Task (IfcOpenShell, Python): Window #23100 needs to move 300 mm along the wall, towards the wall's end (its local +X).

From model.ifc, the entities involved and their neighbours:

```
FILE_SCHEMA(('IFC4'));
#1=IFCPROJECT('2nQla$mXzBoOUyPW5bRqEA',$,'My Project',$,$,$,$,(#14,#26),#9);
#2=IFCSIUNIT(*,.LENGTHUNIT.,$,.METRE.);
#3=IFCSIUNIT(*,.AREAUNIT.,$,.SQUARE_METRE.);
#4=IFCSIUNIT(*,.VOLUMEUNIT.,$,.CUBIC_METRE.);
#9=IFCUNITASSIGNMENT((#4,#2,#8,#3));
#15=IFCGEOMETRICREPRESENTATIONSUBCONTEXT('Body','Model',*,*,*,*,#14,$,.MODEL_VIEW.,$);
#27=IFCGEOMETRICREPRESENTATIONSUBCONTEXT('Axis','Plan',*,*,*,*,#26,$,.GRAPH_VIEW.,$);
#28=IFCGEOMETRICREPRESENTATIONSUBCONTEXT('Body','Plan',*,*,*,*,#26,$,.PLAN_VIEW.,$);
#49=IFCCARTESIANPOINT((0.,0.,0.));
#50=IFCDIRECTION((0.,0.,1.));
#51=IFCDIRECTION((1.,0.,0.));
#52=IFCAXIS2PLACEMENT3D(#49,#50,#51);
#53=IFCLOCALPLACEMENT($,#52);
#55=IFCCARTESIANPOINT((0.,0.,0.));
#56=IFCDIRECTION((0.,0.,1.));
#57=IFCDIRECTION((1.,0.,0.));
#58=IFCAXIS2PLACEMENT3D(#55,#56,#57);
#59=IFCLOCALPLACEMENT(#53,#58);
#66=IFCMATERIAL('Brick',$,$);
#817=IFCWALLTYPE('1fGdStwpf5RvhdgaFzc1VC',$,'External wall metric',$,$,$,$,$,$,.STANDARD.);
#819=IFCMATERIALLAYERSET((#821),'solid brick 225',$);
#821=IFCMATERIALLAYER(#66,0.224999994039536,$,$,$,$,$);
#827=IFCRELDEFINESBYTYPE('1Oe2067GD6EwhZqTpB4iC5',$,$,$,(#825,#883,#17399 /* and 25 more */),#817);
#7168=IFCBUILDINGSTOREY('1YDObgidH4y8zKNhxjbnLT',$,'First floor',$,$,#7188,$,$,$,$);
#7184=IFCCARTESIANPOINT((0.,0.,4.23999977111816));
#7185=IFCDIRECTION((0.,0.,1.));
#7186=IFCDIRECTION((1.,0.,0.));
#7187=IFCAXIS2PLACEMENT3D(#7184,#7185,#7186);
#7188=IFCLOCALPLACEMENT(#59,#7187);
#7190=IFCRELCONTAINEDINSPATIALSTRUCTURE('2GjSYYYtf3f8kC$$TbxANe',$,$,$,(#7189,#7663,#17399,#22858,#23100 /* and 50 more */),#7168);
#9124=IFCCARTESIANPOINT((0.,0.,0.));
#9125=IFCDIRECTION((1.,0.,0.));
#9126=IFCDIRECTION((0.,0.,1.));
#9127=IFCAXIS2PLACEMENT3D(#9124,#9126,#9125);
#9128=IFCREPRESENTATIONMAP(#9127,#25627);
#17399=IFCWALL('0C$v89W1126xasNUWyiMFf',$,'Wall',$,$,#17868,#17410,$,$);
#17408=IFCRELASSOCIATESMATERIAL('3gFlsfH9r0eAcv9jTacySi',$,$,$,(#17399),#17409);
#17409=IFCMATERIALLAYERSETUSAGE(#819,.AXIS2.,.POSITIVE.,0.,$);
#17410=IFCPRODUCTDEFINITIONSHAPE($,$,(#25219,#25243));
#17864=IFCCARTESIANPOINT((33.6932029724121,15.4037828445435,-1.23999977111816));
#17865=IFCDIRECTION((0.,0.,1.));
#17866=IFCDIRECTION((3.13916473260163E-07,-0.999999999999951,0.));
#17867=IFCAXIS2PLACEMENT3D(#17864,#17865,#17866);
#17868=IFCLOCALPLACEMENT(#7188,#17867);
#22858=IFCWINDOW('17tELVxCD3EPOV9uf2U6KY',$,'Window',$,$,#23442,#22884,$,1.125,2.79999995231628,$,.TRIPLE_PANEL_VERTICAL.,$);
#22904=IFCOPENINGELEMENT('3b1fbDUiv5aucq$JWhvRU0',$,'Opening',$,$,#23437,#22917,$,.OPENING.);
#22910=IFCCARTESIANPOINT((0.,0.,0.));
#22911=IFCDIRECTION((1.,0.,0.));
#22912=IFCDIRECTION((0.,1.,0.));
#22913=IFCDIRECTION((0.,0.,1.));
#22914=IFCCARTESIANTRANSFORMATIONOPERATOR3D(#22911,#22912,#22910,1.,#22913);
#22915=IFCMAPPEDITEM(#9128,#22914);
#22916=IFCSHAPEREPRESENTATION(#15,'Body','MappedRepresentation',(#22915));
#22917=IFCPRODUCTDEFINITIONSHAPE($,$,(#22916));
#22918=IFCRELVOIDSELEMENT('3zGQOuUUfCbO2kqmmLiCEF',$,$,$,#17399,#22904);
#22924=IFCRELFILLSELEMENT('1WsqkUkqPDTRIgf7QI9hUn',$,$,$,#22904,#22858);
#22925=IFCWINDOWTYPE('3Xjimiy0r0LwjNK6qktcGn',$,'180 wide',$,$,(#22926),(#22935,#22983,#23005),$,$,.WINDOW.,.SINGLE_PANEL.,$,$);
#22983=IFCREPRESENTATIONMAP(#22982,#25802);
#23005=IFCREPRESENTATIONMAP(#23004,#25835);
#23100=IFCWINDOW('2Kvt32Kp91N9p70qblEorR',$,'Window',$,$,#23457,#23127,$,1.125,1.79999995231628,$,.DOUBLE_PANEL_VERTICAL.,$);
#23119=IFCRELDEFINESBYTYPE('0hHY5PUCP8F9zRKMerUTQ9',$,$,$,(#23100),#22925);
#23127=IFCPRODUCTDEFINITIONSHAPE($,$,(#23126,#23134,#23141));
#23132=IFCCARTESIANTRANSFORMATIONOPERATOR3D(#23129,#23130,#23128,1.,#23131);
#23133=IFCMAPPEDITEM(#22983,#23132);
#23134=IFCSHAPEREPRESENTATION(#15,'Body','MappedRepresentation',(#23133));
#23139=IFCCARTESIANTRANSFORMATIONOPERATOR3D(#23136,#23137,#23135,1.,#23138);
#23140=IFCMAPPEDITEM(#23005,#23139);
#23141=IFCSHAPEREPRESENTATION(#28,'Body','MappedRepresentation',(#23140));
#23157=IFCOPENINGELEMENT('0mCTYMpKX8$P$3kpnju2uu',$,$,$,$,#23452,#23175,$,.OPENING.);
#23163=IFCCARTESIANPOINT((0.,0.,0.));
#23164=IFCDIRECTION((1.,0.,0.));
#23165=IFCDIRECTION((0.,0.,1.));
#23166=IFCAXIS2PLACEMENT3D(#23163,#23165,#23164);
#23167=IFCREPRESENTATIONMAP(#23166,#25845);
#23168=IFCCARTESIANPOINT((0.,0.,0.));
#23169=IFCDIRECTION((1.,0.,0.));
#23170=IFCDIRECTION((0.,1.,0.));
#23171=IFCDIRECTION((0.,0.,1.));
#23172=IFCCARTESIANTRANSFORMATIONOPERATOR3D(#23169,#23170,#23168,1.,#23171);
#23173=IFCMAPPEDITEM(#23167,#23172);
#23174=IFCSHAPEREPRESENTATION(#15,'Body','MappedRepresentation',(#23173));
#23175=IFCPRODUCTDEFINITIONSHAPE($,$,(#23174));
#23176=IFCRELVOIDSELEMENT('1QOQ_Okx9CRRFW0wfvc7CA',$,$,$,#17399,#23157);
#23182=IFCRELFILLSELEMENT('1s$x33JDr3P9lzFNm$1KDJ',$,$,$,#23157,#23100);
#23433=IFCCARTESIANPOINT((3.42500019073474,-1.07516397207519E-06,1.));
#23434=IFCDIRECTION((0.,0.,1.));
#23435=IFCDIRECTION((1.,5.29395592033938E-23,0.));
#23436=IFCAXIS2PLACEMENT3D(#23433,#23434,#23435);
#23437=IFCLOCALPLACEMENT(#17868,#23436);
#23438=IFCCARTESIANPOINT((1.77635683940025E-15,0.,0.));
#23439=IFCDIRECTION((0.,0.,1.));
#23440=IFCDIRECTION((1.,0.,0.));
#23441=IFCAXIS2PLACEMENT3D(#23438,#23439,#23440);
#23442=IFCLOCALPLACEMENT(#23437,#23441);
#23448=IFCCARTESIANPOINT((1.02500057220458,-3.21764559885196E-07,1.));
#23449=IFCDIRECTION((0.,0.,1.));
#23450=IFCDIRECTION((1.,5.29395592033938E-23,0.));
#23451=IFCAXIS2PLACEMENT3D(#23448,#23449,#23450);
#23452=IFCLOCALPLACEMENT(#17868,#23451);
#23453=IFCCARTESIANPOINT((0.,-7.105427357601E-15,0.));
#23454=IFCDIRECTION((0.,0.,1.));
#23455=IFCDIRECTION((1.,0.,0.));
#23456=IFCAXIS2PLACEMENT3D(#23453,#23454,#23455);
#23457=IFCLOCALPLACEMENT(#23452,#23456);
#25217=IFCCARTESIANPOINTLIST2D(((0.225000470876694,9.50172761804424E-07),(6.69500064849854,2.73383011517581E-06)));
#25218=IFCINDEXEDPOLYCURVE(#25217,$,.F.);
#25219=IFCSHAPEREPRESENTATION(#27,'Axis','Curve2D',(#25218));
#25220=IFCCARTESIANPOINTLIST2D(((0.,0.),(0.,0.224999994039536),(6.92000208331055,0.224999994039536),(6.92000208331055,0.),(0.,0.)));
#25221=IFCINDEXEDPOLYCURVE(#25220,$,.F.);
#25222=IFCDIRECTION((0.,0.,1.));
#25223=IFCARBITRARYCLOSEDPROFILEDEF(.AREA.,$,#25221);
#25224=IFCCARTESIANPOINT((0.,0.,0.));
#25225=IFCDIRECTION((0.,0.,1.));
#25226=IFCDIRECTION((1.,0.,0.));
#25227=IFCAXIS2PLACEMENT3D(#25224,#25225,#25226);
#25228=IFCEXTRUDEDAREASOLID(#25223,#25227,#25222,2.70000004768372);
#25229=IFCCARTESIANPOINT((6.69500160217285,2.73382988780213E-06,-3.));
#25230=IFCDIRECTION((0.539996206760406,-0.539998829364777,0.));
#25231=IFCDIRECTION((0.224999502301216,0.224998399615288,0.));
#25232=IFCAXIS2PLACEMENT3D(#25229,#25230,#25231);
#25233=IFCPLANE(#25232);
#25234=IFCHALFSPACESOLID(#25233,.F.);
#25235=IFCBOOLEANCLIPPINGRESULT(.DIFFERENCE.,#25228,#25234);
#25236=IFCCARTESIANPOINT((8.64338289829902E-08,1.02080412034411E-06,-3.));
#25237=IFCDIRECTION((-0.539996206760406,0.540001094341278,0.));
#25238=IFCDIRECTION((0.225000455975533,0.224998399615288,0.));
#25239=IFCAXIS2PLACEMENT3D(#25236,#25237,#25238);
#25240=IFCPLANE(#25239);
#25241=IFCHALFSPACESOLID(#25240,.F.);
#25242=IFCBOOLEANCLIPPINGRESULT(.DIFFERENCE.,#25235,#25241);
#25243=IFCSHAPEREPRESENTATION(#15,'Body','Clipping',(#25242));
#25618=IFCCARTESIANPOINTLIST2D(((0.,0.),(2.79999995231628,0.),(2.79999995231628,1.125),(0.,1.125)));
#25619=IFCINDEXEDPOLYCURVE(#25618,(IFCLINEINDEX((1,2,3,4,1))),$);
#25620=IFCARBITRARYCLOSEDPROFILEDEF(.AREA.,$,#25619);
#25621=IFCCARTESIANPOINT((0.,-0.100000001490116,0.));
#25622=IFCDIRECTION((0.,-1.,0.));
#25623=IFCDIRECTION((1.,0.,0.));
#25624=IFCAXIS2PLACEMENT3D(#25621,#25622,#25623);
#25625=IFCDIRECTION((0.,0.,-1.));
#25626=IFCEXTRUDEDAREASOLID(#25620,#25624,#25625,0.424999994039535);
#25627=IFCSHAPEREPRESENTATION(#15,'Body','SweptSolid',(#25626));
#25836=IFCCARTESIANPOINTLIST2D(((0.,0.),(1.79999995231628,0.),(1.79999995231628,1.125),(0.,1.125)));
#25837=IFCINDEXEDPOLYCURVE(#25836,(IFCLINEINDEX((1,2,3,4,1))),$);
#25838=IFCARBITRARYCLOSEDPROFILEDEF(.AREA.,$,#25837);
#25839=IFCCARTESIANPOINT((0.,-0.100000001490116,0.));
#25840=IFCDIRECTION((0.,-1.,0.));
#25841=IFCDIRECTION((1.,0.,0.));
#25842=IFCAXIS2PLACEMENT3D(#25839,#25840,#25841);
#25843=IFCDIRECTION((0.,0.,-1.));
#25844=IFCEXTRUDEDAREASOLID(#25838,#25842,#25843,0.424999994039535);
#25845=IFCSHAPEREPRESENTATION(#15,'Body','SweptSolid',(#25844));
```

```python
import ifcopenshell
import ifcopenshell.api.geometry
import ifcopenshell.util.placement
import ifcopenshell.util.unit

model = ifcopenshell.open("model.ifc")
unit_scale = ifcopenshell.util.unit.calculate_unit_scale(model)

window = model.by_id(23100)
opening = window.FillsVoids[0].RelatingOpeningElement
wall = opening.VoidsElements[0].RelatingBuildingElement

wall_matrix = ifcopenshell.util.placement.get_local_placement(wall.ObjectPlacement)
shift = wall_matrix[:3, 0] * 0.3 / unit_scale
before = ifcopenshell.util.placement.get_local_placement(window.ObjectPlacement)[:3, 3].copy()

# The window is placed relative to its opening, so it follows when the opening moves.
matrix = ifcopenshell.util.placement.get_local_placement(opening.ObjectPlacement)
matrix[:3, 3] += shift
ifcopenshell.api.geometry.edit_object_placement(
    model, product=opening, matrix=matrix, is_si=False, should_transform_children=True
)

after = ifcopenshell.util.placement.get_local_placement(window.ObjectPlacement)[:3, 3]
print("window moved by", (after - before).round(3) + 0.0)

model.write("model_v2.ifc")
```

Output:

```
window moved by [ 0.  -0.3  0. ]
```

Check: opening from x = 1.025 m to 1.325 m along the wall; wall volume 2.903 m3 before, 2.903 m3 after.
